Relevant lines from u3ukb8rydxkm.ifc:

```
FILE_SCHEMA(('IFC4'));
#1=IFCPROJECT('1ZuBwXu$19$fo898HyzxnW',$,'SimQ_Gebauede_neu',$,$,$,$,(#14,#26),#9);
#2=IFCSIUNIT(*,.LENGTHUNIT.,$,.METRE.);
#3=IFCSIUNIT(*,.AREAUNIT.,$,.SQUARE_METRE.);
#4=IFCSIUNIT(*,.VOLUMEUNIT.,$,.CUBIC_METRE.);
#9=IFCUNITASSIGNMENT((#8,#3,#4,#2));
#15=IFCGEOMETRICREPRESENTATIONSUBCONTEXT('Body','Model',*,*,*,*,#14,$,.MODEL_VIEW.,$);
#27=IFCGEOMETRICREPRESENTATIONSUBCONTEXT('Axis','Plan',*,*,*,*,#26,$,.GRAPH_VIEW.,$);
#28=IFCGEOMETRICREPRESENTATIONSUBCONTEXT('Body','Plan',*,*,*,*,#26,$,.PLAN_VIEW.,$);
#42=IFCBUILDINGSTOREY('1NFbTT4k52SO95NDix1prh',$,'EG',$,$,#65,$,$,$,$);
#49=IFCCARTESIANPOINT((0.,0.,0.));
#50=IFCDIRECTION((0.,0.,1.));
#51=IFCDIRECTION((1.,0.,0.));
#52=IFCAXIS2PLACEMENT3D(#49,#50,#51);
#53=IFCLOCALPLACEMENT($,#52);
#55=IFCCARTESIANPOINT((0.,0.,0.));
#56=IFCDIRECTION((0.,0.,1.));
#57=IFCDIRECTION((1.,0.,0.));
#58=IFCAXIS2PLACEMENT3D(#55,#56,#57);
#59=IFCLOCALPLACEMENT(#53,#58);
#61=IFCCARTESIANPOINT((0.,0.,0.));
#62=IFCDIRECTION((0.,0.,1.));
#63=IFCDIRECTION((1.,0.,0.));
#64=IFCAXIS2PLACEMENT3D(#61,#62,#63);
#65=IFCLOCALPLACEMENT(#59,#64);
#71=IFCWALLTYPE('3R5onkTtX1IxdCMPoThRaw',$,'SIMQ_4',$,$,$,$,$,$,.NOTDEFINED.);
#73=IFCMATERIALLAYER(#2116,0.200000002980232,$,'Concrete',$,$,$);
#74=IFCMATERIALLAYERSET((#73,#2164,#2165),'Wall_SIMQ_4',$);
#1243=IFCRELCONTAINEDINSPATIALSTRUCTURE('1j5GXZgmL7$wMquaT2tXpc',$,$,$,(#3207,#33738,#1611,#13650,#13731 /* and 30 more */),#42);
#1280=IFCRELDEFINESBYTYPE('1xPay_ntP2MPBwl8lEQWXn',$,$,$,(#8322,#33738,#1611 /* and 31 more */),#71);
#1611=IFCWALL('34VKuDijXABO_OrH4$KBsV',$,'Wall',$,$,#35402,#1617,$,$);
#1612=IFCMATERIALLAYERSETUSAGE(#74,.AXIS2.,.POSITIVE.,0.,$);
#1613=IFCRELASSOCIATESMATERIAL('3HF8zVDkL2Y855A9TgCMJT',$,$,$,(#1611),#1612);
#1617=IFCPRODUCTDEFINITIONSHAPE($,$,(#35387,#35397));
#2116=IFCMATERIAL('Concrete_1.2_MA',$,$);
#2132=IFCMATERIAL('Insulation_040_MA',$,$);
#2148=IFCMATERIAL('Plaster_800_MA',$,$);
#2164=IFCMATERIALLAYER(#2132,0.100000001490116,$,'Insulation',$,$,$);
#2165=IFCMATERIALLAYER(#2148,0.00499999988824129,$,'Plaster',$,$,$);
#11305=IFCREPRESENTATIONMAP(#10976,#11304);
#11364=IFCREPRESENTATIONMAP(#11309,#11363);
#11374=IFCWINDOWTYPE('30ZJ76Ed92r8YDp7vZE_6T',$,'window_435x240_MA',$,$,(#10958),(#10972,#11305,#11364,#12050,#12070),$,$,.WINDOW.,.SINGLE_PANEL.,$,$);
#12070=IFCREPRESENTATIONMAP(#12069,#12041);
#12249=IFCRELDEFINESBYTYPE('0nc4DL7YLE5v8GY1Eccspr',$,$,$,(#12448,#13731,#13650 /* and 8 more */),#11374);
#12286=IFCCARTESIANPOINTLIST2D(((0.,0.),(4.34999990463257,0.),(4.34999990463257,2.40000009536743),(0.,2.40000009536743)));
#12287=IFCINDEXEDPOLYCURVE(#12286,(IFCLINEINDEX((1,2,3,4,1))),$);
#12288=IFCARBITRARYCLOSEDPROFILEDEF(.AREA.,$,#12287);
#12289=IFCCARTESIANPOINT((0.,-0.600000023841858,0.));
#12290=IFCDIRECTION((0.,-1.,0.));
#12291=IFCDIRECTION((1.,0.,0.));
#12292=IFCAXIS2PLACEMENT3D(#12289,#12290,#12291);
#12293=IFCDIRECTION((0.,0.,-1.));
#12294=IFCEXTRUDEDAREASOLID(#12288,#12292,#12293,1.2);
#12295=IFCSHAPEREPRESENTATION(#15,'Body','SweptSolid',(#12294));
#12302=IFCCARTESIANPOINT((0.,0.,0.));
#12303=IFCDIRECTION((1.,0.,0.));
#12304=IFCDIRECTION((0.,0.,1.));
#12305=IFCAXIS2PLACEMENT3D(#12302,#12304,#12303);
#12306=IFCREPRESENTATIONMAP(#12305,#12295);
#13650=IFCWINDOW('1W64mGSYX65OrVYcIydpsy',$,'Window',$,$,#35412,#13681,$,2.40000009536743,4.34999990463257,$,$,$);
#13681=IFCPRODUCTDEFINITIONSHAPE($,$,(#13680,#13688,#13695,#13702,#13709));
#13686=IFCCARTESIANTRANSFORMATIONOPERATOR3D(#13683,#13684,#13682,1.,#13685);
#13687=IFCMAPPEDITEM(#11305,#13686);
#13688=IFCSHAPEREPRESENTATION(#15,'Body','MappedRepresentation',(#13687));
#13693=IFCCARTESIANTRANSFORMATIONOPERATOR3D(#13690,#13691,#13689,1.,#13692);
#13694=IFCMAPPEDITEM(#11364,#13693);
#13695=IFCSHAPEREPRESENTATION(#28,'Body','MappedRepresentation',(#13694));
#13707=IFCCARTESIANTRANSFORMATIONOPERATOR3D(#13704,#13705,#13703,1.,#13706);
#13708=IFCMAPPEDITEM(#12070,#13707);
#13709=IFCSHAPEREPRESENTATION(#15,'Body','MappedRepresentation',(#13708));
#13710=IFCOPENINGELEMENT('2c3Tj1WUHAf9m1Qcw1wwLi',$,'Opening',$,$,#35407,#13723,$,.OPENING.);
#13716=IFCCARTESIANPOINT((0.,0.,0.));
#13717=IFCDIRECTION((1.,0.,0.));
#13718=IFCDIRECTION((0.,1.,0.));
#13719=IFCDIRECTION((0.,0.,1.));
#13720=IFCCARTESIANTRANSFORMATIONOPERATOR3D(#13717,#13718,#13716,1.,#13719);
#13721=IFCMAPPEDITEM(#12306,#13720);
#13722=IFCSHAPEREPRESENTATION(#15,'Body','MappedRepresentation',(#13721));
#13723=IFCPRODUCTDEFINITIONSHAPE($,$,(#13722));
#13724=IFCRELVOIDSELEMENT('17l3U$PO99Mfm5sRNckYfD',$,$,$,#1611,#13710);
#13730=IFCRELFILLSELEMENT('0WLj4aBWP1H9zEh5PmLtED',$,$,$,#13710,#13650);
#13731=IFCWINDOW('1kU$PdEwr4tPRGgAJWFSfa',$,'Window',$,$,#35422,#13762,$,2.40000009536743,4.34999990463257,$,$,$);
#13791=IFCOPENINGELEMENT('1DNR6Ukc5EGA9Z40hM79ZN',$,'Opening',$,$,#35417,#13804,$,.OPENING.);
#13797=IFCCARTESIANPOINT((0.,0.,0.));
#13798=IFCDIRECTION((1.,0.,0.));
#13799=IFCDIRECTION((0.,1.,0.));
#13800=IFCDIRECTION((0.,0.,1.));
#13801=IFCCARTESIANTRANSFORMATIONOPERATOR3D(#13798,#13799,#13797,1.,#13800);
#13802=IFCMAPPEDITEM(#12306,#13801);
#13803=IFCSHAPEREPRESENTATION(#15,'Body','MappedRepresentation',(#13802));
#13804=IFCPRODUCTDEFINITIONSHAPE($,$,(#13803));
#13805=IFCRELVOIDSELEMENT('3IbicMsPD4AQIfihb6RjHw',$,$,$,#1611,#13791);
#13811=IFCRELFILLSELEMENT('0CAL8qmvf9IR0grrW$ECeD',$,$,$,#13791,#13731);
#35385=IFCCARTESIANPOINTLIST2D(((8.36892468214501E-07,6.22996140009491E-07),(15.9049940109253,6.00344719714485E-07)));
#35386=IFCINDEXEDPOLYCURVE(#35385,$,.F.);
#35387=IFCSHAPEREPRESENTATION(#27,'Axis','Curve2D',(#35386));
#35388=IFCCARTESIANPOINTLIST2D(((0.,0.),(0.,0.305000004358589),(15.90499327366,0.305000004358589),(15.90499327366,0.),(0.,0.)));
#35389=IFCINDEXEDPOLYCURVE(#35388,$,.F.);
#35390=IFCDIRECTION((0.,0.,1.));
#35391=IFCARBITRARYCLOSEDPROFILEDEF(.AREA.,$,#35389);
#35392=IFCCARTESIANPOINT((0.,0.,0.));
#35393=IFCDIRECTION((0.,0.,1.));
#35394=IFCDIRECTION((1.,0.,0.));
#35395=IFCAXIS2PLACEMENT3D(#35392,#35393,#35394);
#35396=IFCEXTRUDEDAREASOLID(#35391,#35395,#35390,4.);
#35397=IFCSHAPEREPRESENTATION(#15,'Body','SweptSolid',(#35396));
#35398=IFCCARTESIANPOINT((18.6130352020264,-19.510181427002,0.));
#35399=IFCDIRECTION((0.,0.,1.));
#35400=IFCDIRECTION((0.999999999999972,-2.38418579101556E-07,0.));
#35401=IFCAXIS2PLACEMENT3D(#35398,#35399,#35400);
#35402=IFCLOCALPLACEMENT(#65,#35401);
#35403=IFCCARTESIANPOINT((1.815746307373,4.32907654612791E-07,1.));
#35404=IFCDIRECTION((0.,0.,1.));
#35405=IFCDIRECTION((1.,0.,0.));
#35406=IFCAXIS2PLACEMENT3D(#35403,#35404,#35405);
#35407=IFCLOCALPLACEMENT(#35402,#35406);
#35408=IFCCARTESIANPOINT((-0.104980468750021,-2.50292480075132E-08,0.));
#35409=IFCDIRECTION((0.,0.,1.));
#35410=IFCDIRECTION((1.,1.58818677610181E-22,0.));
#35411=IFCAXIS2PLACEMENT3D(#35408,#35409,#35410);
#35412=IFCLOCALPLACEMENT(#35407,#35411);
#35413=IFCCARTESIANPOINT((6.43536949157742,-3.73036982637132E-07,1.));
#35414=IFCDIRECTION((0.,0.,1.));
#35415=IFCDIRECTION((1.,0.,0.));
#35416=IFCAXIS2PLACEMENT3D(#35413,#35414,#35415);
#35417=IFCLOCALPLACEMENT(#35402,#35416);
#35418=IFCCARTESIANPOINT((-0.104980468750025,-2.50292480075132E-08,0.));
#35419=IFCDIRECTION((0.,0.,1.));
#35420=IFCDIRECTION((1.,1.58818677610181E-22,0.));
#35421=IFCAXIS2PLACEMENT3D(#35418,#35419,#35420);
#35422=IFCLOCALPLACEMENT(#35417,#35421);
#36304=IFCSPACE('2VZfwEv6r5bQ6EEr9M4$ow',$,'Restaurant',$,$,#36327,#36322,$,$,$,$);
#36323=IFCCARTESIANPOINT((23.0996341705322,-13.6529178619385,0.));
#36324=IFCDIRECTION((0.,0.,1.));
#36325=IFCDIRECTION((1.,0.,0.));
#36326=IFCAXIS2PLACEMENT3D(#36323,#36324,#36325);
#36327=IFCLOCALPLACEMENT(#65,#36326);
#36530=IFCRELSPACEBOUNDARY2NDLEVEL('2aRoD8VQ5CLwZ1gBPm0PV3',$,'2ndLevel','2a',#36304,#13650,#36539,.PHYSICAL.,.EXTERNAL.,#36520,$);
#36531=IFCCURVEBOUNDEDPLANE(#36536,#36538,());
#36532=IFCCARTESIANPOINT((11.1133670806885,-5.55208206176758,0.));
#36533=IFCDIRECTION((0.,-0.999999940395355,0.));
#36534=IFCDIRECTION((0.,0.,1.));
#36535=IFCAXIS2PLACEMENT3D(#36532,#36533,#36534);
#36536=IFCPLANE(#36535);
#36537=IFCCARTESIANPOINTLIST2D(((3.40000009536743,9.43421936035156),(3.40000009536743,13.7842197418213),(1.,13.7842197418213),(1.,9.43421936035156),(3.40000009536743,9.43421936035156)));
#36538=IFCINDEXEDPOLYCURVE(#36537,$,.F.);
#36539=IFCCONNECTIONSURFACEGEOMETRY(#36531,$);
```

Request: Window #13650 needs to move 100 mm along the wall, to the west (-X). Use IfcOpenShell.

```python
import numpy as np
import ifcopenshell
import ifcopenshell.api.geometry
import ifcopenshell.util.placement

model = ifcopenshell.open("u3ukb8rydxkm.ifc")

window = model.by_id(13650)
opening = window.FillsVoids[0].RelatingOpeningElement
wall = opening.VoidsElements[0].RelatingBuildingElement

wall_matrix = ifcopenshell.util.placement.get_local_placement(wall.ObjectPlacement)
shift = wall_matrix[:3, 0] * -0.1
before = ifcopenshell.util.placement.get_local_placement(window.ObjectPlacement)[:3, 3].copy()

# The window is placed relative to its opening, so it follows when the opening moves.
matrix = ifcopenshell.util.placement.get_local_placement(opening.ObjectPlacement)
matrix[:3, 3] += shift
ifcopenshell.api.geometry.edit_object_placement(
    model, product=opening, matrix=matrix, is_si=False, should_transform_children=True
)

# Space boundary surfaces are stored in each space's coordinates; move them too.
for rel in window.ProvidesBoundaries:
    if not rel.ConnectionGeometry:
        continue
    surface = rel.ConnectionGeometry.SurfaceOnRelatingElement.BasisSurface
    space_matrix = ifcopenshell.util.placement.get_local_placement(rel.RelatingSpace.ObjectPlacement)
    point = np.array(surface.Position.Location.Coordinates) + space_matrix[:3, :3].T @ shift
    surface.Position = model.createIfcAxis2Placement3D(
        model.createIfcCartesianPoint(point.tolist()), surface.Position.Axis, surface.Position.RefDirection
    )

after = ifcopenshell.util.placement.get_local_placement(window.ObjectPlacement)[:3, 3]
print("window moved by", (after - before).round(3) + 0.0)

model.write("u3ukb8rydxkm_updated.ifc")
```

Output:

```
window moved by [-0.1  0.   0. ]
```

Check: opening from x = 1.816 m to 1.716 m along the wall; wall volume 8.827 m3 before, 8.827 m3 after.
